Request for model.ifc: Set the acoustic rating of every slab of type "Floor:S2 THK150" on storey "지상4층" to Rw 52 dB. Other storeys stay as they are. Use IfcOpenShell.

First a look at what the model holds.

```python
import ifcopenshell
import ifcopenshell.util.element

model = ifcopenshell.open("model.ifc")
print(model.schema)
storey = next(s for s in model.by_type("IfcBuildingStorey") if s.Name == "지상4층")
slabs = [e for e in ifcopenshell.util.element.get_decomposition(storey) if e.is_a("IfcSlab")]
seen = {}
for e in slabs:
    element_type = ifcopenshell.util.element.get_type(e)
    key = (element_type.Name if element_type != e and element_type else None, ifcopenshell.util.element.get_pset(e, "Pset_SlabCommon", "AcousticRating"))
    seen[key] = seen.get(key, 0) + 1
for (name, value), count in sorted(seen.items(), key=str):
    print(count, "x", name, "|", value)
```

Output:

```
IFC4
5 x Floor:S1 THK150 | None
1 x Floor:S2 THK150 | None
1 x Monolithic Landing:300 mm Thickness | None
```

```python
import ifcopenshell
import ifcopenshell.api.pset
import ifcopenshell.util.element

model = ifcopenshell.open("model.ifc")

storey = next(s for s in model.by_type("IfcBuildingStorey") if s.Name == "지상4층")
slabs = [e for e in ifcopenshell.util.element.get_decomposition(storey) if e.is_a("IfcSlab")]

count = 0
for e in slabs:
    element_type = ifcopenshell.util.element.get_type(e)
    if element_type in (None, e) or element_type.Name != "Floor:S2 THK150":
        continue
    # add_pset returns the element's existing set when there is one.
    pset = ifcopenshell.api.pset.add_pset(model, product=e, name="Pset_SlabCommon")
    ifcopenshell.api.pset.edit_pset(model, pset=pset, properties={"AcousticRating": "Rw 52 dB"})
    count += 1

print(count, "slabs updated")

model.write("model_edited.ifc")
```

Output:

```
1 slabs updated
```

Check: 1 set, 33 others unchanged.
